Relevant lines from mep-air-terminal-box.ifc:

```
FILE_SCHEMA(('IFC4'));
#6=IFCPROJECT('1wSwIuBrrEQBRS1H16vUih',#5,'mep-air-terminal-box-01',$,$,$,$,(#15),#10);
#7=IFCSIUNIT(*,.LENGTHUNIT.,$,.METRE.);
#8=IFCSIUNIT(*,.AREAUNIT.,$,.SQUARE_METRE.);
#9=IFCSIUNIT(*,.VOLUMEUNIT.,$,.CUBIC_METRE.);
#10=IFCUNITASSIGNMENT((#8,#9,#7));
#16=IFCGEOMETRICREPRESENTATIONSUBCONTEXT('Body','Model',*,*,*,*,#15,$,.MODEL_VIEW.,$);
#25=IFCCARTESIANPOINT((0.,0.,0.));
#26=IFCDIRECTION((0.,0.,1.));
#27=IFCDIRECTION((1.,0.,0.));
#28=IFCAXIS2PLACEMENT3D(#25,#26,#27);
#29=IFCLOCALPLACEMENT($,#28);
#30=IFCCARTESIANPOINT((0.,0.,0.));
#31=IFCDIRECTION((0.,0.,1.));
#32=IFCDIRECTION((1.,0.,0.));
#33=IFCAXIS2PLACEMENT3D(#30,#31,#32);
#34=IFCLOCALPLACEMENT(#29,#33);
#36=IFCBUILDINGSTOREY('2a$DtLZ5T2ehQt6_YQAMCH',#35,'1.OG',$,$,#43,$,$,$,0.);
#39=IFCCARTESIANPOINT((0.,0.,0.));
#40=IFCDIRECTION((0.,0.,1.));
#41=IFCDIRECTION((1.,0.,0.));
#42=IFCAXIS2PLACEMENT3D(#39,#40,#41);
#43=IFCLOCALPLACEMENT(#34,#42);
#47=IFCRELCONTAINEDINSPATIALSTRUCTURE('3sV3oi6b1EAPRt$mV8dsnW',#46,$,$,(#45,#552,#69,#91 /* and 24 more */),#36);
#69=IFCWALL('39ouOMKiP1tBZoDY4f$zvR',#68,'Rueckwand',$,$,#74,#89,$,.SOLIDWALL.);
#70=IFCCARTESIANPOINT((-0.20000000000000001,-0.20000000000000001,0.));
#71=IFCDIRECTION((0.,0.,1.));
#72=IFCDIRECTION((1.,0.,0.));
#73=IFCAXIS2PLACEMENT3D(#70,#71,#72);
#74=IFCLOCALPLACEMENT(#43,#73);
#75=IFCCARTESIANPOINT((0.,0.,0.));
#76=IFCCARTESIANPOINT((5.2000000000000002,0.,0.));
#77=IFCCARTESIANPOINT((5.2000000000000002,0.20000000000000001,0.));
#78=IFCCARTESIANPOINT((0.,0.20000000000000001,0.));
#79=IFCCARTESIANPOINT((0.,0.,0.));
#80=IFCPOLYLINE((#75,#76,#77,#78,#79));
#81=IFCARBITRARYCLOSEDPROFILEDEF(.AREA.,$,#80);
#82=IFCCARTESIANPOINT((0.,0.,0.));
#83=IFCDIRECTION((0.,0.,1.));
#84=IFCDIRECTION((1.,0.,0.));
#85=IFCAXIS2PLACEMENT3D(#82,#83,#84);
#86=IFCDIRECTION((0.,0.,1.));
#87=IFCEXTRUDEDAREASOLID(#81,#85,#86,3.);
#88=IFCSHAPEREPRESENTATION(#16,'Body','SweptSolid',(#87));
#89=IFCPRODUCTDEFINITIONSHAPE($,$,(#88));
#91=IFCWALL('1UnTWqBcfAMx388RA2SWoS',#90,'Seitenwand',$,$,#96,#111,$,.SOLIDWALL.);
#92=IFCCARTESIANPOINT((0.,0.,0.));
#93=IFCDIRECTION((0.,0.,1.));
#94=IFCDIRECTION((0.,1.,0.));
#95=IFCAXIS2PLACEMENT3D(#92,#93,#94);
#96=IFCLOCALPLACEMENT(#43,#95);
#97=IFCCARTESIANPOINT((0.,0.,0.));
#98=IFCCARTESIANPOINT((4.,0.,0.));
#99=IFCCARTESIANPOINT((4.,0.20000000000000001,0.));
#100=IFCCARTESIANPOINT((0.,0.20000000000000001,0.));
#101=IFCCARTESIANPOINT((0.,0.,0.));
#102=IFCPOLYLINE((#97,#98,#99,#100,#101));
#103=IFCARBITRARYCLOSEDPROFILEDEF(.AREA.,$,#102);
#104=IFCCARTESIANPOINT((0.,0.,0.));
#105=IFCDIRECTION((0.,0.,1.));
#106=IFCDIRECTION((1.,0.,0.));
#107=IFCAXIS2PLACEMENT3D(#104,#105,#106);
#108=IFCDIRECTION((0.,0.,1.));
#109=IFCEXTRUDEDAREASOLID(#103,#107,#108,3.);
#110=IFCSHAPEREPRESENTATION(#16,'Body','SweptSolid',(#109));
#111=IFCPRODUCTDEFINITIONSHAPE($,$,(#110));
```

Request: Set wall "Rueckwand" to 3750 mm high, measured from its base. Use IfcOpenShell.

```python
import ifcopenshell
import ifcopenshell.geom
import ifcopenshell.util.representation
import ifcopenshell.util.shape
import ifcopenshell.util.unit

model = ifcopenshell.open("mep-air-terminal-box.ifc")
unit_scale = ifcopenshell.util.unit.calculate_unit_scale(model)
settings = ifcopenshell.geom.settings()


def volume(element):
    """Net volume in cubic metres, openings subtracted."""
    shape = ifcopenshell.geom.create_shape(settings, element)
    return ifcopenshell.util.shape.get_volume(shape.geometry)


wall = model.by_guid("39ouOMKiP1tBZoDY4f$zvR")
before = volume(wall)

body = ifcopenshell.util.representation.get_representation(wall, "Model", "Body")
solid = body.Items[0]
old_height = solid.Depth
solid.Depth = 3.75 / unit_scale
after = volume(wall)

print(f"height {old_height:g} -> {solid.Depth:g}, volume {before:.3f} -> {after:.3f} m3")

model.write("mep-air-terminal-box_v2.ifc")
```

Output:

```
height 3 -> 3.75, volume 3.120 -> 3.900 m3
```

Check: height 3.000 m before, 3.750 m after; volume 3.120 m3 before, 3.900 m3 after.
